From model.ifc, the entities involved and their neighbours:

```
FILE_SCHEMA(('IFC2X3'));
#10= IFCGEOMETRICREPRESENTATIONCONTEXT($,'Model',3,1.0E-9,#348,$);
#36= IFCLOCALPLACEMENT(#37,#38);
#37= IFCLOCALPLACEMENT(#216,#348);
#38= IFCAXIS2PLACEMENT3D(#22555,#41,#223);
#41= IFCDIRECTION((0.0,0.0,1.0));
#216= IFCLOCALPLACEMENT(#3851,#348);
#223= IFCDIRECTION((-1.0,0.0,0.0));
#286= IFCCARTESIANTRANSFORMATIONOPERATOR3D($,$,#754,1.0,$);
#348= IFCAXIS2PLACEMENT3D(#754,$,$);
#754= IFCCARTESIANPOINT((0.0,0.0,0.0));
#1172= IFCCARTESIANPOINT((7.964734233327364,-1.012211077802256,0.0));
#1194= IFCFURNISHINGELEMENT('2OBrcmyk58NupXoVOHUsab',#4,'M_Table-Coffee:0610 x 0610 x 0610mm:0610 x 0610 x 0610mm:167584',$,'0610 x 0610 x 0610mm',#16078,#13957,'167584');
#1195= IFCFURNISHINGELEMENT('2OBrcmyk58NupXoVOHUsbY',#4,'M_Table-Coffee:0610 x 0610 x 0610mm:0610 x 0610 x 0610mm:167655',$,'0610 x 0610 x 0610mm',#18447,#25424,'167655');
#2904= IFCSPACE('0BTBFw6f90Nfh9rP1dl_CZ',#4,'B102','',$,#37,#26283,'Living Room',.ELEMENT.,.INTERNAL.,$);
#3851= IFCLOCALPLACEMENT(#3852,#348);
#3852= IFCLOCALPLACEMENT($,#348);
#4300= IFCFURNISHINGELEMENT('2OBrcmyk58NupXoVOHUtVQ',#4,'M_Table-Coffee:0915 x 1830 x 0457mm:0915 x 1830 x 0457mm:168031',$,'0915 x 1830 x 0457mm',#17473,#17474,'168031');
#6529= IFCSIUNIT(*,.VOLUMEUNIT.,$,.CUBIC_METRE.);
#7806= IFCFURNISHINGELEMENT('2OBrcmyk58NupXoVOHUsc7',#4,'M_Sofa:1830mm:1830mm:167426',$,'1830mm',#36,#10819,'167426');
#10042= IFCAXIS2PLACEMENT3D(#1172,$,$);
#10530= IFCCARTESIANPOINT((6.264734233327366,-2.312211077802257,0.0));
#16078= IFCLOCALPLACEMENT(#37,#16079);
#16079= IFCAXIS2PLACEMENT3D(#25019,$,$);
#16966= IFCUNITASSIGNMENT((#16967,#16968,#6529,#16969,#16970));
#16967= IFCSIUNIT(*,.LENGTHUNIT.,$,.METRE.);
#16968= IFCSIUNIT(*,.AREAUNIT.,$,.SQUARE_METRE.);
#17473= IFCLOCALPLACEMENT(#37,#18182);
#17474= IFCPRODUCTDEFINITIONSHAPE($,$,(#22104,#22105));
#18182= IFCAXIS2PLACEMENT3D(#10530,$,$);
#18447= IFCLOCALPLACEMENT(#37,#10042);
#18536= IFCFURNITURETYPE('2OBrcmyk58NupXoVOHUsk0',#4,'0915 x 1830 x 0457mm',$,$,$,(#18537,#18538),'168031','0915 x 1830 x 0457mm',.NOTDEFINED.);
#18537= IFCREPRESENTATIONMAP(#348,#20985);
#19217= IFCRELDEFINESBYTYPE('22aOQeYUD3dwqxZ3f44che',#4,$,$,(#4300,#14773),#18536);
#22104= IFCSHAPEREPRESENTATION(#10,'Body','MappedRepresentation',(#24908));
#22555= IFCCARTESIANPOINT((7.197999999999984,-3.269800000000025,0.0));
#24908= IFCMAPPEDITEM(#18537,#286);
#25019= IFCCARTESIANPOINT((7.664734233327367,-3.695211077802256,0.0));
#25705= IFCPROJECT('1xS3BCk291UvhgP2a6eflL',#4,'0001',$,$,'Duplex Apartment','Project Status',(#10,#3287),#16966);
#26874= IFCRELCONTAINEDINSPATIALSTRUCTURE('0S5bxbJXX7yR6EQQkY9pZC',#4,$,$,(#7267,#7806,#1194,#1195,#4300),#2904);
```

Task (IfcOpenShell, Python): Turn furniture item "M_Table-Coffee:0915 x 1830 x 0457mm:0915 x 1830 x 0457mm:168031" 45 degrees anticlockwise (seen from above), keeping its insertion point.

```python
import ifcopenshell
import ifcopenshell.api.geometry
import ifcopenshell.util.placement

model = ifcopenshell.open("model.ifc")

item = model.by_id(4300)
matrix = ifcopenshell.util.placement.get_local_placement(item.ObjectPlacement)
matrix = matrix @ ifcopenshell.util.placement.rotation(45, "Z")
ifcopenshell.api.geometry.edit_object_placement(model, product=item, matrix=matrix, is_si=False)

print(ifcopenshell.util.placement.get_local_placement(item.ObjectPlacement).round(3) + 0.0)

model.write("model_rev.ifc")
```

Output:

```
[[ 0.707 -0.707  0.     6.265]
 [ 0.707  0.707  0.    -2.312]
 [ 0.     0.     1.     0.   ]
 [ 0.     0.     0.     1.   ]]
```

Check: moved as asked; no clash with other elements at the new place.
